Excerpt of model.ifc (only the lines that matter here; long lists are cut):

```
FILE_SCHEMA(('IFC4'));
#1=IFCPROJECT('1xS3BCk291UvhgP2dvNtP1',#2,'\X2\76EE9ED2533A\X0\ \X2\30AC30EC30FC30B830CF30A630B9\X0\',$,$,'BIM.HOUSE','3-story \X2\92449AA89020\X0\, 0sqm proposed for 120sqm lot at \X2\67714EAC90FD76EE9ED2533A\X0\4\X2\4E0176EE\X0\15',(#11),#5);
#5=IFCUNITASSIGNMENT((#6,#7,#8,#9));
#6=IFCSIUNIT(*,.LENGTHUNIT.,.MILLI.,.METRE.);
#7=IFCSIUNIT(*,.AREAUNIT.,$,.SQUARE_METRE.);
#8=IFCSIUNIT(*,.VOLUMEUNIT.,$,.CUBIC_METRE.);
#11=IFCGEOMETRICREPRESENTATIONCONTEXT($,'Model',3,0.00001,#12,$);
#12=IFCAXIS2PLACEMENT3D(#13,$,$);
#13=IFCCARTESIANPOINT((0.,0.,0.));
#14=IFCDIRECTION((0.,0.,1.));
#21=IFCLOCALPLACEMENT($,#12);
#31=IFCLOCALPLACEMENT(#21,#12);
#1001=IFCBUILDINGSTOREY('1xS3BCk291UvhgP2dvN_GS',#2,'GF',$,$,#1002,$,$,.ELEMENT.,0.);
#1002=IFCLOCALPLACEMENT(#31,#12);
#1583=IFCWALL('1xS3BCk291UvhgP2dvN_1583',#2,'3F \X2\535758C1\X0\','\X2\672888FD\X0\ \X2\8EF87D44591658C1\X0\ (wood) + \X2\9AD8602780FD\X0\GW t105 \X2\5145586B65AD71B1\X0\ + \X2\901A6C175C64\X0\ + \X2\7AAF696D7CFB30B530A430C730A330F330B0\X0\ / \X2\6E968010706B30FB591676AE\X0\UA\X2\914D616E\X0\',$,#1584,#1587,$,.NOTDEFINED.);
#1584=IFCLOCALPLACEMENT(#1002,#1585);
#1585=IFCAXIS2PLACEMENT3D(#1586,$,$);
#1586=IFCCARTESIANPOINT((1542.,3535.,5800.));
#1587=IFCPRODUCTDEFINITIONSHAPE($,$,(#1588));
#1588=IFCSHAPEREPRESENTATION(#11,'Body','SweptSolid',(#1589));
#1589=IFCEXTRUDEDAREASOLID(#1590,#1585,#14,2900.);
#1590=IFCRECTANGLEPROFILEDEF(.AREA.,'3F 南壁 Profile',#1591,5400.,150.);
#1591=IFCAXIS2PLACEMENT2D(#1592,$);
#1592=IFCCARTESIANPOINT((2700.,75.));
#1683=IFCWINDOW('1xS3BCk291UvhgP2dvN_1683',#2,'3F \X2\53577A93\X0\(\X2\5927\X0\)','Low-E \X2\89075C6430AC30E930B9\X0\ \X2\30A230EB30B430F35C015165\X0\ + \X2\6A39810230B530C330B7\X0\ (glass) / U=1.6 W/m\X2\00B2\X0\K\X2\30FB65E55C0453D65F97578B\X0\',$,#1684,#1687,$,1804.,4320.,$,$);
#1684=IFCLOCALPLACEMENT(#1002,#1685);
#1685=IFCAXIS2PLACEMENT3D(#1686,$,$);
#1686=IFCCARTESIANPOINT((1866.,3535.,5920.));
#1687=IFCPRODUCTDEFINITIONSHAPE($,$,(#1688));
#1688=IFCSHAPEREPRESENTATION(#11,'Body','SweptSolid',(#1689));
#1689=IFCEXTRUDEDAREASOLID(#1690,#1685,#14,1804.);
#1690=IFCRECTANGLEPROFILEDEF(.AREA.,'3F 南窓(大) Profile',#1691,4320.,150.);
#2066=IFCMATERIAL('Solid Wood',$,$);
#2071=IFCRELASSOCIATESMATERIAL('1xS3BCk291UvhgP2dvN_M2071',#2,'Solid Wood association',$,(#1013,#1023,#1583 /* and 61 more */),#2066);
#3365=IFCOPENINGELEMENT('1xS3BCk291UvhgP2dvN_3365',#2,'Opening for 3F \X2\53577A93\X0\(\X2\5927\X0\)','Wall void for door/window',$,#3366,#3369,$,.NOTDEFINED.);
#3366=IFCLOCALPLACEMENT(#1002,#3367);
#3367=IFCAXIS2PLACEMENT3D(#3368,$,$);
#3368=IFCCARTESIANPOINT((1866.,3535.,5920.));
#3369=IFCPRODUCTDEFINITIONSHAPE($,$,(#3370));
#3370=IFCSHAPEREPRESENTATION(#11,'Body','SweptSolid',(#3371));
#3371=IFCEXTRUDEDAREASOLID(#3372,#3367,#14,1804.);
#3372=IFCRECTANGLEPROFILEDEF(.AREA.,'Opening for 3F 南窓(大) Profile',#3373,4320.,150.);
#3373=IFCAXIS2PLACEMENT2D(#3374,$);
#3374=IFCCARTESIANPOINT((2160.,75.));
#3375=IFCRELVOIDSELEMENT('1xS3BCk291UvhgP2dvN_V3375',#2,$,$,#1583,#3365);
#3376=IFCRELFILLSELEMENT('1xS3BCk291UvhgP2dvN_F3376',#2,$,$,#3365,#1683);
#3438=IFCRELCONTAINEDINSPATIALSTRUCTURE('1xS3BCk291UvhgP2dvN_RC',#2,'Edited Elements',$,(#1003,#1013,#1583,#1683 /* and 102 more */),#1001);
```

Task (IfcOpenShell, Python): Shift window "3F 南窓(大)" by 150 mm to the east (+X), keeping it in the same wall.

```python
import ifcopenshell
import ifcopenshell.api.geometry
import ifcopenshell.util.placement
import ifcopenshell.util.unit

model = ifcopenshell.open("model.ifc")
unit_scale = ifcopenshell.util.unit.calculate_unit_scale(model)

window = model.by_guid("1xS3BCk291UvhgP2dvN_1683")
opening = window.FillsVoids[0].RelatingOpeningElement
wall = opening.VoidsElements[0].RelatingBuildingElement

wall_matrix = ifcopenshell.util.placement.get_local_placement(wall.ObjectPlacement)
shift = wall_matrix[:3, 0] * 0.15 / unit_scale
before = ifcopenshell.util.placement.get_local_placement(window.ObjectPlacement)[:3, 3].copy()

# The window is not placed relative to its opening, so move both.
for product in (opening, window):
    matrix = ifcopenshell.util.placement.get_local_placement(product.ObjectPlacement)
    matrix[:3, 3] += shift
    ifcopenshell.api.geometry.edit_object_placement(model, product=product, matrix=matrix, is_si=False)

after = ifcopenshell.util.placement.get_local_placement(window.ObjectPlacement)[:3, 3]
print("window moved by", (after - before).round(3) + 0.0)

model.write("model_rev.ifc")
```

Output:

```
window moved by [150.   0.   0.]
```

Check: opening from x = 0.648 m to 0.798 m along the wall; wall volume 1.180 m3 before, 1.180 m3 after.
